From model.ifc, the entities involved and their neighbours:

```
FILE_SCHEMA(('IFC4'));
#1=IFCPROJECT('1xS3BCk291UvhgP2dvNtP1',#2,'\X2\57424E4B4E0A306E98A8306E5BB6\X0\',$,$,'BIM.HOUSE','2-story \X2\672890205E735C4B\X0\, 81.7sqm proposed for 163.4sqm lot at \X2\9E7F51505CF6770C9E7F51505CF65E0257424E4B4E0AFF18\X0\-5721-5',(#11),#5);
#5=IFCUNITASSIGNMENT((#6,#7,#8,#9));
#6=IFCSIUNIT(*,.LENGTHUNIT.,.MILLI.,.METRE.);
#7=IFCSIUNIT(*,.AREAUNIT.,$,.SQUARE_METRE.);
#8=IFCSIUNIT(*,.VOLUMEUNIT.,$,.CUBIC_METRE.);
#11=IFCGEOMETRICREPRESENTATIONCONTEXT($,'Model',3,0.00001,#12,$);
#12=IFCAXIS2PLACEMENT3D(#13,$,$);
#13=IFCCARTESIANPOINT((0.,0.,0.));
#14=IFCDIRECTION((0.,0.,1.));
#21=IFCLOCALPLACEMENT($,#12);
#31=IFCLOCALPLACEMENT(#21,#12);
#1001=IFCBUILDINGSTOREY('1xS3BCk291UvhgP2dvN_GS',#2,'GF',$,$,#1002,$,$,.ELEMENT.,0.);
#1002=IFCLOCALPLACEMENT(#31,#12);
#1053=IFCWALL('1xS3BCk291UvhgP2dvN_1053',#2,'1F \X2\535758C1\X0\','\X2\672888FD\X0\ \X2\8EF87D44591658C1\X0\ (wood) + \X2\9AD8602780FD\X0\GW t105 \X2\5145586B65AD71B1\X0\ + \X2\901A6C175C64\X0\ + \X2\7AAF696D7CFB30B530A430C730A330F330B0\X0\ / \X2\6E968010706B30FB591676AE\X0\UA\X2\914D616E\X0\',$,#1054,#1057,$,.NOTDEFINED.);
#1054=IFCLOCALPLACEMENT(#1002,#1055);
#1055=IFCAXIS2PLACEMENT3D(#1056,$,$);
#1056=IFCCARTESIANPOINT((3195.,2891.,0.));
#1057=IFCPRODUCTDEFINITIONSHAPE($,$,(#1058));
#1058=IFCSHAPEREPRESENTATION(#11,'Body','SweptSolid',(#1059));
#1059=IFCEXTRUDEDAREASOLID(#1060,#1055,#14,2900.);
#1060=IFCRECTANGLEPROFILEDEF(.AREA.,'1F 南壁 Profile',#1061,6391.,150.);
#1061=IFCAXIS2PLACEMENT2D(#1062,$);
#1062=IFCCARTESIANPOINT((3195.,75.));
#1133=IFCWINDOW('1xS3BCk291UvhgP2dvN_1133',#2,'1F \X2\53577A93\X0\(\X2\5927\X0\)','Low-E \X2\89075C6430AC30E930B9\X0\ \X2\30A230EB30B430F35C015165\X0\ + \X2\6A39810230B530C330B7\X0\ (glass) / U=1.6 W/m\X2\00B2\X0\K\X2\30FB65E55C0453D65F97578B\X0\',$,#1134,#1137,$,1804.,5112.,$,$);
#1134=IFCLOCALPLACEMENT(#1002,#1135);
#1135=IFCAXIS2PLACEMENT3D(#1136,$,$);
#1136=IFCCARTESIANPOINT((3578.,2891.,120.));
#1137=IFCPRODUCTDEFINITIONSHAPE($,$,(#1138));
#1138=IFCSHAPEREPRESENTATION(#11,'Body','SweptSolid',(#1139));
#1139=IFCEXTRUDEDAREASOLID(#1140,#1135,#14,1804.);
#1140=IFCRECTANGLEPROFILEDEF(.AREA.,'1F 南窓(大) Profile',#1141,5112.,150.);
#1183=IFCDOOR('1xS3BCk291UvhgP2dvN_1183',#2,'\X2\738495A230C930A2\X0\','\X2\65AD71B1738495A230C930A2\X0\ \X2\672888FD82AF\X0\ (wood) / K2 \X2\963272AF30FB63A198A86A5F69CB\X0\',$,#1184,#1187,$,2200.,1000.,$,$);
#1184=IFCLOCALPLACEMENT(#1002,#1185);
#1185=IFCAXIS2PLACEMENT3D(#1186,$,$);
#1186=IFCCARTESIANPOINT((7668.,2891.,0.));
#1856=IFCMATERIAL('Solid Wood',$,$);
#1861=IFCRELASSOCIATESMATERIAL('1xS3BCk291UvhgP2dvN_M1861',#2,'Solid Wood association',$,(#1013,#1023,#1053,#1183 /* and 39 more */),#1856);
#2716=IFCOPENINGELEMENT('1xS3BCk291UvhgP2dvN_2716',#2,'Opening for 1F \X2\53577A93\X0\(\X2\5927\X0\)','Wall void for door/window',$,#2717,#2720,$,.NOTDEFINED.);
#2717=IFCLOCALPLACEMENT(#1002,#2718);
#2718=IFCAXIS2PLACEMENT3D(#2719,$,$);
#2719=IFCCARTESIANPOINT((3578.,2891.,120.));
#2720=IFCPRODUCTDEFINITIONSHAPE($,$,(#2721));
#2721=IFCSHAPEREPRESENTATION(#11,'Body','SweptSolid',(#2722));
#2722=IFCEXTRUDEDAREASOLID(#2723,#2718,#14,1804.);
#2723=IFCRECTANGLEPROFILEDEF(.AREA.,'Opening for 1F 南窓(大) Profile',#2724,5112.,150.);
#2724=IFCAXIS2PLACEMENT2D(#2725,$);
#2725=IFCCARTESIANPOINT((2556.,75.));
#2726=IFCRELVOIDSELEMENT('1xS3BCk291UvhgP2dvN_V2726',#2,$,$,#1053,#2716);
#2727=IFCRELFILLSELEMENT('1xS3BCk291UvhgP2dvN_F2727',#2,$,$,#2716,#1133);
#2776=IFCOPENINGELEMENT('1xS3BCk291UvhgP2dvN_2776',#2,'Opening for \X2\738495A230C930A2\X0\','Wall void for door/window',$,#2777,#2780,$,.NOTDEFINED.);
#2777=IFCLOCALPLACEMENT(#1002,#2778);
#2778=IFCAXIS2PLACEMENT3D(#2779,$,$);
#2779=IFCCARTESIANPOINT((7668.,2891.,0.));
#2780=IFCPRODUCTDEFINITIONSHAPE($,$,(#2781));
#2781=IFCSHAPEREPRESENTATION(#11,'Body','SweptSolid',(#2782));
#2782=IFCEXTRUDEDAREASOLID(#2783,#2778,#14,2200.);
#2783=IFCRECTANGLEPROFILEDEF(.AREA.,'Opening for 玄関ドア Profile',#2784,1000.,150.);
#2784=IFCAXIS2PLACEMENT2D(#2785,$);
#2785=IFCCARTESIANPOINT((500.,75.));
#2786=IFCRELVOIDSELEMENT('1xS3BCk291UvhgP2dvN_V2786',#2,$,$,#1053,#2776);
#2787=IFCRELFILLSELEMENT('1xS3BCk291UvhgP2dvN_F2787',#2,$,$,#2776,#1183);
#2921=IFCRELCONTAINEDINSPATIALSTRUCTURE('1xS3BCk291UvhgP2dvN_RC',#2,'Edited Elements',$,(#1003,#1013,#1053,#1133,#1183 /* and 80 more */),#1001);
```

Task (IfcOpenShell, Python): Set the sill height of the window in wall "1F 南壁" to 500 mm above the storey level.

```python
import numpy as np
import ifcopenshell
import ifcopenshell.api.geometry
import ifcopenshell.geom
import ifcopenshell.util.element
import ifcopenshell.util.placement
import ifcopenshell.util.shape
import ifcopenshell.util.unit

model = ifcopenshell.open("model.ifc")
unit_scale = ifcopenshell.util.unit.calculate_unit_scale(model)

window = model.by_guid("1xS3BCk291UvhgP2dvN_1133")
opening = window.FillsVoids[0].RelatingOpeningElement
storey = ifcopenshell.util.element.get_container(window, ifc_class="IfcBuildingStorey")
level = ifcopenshell.util.placement.get_local_placement(storey.ObjectPlacement)[2, 3]

# The opening's origin need not be at the sill, so measure its lowest point.
shape = ifcopenshell.geom.create_shape(ifcopenshell.geom.settings(), opening)
bottom = ifcopenshell.util.shape.get_shape_bottom_elevation(shape, shape.geometry) / unit_scale
dz = level + 500.0 - bottom

shift = np.array([0.0, 0.0, dz])
# The window is not placed relative to its opening, so move both.
for product in (opening, window):
    matrix = ifcopenshell.util.placement.get_local_placement(product.ObjectPlacement)
    matrix[:3, 3] += shift
    ifcopenshell.api.geometry.edit_object_placement(model, product=product, matrix=matrix, is_si=False)

print(f"moved by {dz * unit_scale:+.3f} m")

model.write("model_v2.ifc")
```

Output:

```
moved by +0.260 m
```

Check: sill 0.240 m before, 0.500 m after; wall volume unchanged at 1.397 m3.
